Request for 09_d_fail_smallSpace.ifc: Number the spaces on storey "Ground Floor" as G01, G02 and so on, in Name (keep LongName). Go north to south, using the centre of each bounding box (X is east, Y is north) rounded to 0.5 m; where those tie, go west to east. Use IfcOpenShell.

First a look at what the model holds.

```python
import ifcopenshell
import ifcopenshell.util.element
import ifcopenshell.util.placement

model = ifcopenshell.open("09_d_fail_smallSpace.ifc")
print(model.schema)
storey = next(s for s in model.by_type("IfcBuildingStorey") if s.Name == "Ground Floor")
spaces = [e for e in ifcopenshell.util.element.get_decomposition(storey) if e.is_a("IfcSpace")]
for e in sorted(spaces, key=lambda e: e.id()):
    origin = ifcopenshell.util.placement.get_local_placement(e.ObjectPlacement)[:3, 3]
    print(e.id(), e.Name, e.LongName, origin.round(2) + 0.0, sep=" | ")
```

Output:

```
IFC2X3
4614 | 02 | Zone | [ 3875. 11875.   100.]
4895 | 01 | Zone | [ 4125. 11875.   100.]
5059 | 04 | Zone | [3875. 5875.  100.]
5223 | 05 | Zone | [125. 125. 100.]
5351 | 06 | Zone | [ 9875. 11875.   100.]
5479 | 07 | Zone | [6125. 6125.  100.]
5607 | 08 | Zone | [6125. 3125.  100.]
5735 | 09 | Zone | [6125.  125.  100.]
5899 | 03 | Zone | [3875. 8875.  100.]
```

```python
import ifcopenshell
import ifcopenshell.geom
import ifcopenshell.util.element
import ifcopenshell.util.shape

model = ifcopenshell.open("09_d_fail_smallSpace.ifc")
settings = ifcopenshell.geom.settings()
settings.set("use-world-coords", True)


def centre(element):
    shape = ifcopenshell.geom.create_shape(settings, element)
    return ifcopenshell.util.shape.get_bbox_centroid(shape.geometry)


storey = next(s for s in model.by_type("IfcBuildingStorey") if s.Name == "Ground Floor")
spaces = [e for e in ifcopenshell.util.element.get_decomposition(storey) if e.is_a("IfcSpace")]

# Insertion points can sit at a corner or the storey origin, so sort by the geometry (in metres).
centres = {e: centre(e) for e in spaces}
spaces.sort(key=lambda e: (-round(centres[e][1] / 0.5), centres[e][0]))

for i, e in enumerate(spaces, start=1):
    number = f"G{i:02d}"
    e.Name = number
    print(e.id(), number)

model.write("09_d_fail_smallSpace_rev.ifc")
```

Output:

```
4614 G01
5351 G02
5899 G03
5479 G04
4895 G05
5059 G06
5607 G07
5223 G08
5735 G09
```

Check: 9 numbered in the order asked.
